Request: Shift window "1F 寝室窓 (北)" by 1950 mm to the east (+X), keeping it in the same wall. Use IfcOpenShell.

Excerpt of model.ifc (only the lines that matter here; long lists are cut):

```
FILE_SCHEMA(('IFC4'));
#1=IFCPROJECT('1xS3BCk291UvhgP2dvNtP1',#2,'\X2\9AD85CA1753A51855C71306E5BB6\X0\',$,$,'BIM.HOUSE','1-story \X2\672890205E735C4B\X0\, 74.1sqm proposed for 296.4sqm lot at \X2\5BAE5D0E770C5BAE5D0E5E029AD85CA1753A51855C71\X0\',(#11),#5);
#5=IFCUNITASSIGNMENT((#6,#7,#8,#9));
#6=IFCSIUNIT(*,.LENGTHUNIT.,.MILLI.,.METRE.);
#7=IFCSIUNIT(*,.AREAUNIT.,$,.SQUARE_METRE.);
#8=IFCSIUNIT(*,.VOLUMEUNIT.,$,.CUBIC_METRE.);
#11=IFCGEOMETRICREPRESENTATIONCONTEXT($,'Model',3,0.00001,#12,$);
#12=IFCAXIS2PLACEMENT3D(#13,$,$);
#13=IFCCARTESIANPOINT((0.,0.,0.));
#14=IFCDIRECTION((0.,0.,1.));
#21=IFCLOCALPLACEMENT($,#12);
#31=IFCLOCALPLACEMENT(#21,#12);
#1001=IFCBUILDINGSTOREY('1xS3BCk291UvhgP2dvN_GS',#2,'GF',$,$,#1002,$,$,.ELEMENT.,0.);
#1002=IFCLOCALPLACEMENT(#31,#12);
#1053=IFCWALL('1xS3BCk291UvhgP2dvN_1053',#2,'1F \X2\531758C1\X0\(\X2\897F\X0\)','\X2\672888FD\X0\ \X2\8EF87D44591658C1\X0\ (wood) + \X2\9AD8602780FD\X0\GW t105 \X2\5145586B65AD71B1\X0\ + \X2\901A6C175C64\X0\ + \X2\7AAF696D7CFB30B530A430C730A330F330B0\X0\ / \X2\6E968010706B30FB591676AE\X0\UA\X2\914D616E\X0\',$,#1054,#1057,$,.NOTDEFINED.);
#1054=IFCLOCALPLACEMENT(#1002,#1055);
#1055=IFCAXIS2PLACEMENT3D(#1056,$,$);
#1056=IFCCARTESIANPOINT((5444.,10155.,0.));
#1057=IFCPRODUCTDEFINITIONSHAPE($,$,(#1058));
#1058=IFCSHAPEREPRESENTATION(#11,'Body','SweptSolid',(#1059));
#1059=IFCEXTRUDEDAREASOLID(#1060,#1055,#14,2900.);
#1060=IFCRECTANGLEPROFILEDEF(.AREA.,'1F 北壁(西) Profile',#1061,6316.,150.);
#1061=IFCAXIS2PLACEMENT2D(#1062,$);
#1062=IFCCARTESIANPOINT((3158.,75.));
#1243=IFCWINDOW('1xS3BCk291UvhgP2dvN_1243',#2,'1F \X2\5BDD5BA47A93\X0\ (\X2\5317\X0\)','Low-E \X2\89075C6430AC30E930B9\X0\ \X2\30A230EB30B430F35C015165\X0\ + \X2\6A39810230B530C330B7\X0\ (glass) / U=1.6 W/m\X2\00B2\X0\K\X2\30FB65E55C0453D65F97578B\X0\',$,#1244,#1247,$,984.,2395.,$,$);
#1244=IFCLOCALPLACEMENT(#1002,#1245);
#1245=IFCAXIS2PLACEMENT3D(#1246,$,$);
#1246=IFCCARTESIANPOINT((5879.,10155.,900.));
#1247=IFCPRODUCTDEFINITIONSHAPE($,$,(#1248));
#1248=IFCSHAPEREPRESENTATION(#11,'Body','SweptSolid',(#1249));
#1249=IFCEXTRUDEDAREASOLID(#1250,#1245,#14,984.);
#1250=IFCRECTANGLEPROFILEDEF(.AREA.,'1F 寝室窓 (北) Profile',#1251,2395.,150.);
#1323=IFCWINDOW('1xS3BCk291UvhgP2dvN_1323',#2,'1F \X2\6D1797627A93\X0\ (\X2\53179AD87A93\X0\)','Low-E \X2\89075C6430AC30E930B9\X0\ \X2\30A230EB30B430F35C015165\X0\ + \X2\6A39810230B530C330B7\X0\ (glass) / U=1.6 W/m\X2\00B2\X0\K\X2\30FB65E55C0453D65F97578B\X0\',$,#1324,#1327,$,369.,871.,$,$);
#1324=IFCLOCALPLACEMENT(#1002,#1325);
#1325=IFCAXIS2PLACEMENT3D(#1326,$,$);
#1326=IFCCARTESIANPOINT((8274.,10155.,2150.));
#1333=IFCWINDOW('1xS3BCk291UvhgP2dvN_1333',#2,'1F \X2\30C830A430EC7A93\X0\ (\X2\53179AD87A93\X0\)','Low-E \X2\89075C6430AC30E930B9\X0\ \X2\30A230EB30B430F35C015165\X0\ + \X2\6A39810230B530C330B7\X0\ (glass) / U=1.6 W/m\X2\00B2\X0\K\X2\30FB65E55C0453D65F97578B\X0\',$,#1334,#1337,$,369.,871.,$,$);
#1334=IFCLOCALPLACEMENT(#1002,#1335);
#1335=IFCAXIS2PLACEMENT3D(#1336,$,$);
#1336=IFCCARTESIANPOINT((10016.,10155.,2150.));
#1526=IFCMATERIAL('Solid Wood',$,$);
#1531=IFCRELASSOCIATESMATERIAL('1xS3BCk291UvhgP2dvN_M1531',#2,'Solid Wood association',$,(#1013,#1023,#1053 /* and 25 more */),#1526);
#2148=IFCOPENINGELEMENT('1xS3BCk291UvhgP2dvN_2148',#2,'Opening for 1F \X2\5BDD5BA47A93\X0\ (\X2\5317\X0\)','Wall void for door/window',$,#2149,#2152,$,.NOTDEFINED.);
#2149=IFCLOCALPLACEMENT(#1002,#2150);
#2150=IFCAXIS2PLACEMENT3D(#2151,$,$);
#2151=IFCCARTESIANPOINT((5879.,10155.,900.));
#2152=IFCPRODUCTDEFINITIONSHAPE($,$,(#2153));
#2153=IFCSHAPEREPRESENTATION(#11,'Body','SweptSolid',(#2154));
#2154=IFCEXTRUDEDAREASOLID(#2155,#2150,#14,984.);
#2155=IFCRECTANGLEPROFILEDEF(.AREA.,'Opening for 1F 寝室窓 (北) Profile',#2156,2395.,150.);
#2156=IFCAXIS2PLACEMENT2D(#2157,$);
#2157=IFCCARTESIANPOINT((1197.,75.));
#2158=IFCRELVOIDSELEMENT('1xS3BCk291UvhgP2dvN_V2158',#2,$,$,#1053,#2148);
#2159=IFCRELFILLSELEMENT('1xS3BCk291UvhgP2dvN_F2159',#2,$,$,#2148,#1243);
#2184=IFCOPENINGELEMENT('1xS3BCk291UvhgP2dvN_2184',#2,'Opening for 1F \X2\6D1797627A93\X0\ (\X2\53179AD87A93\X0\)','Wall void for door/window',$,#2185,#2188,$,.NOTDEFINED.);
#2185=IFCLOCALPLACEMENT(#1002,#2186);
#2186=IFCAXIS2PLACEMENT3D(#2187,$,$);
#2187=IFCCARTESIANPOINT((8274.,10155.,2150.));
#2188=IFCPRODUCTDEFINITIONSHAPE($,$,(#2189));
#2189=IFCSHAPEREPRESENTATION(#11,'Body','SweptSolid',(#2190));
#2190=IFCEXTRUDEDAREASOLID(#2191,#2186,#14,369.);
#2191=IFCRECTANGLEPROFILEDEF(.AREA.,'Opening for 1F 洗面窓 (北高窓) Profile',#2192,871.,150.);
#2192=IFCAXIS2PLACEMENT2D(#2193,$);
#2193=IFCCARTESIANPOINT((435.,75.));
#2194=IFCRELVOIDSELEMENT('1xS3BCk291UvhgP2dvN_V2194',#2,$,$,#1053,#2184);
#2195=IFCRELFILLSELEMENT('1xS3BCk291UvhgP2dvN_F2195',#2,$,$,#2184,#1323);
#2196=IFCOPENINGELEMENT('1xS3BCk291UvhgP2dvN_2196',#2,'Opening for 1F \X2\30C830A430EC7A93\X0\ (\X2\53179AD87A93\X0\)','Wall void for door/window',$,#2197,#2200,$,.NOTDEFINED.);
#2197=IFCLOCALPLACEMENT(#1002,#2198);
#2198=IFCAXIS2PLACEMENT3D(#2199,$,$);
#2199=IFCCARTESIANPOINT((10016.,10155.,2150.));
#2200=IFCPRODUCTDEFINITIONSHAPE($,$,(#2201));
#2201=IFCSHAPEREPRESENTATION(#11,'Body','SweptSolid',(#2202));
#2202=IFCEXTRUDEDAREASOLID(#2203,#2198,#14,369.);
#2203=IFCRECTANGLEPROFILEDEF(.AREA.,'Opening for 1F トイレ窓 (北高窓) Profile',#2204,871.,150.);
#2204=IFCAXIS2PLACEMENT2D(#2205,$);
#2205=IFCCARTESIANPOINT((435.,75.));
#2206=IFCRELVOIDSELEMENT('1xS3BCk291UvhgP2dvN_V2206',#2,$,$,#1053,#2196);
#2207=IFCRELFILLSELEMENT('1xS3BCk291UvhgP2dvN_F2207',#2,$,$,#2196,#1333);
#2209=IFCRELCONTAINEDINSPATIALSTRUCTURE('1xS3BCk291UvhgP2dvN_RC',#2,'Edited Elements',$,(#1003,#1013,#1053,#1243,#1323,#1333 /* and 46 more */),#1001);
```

```python
import ifcopenshell
import ifcopenshell.api.geometry
import ifcopenshell.util.placement

model = ifcopenshell.open("model.ifc")

window = model.by_guid("1xS3BCk291UvhgP2dvN_1243")
opening = window.FillsVoids[0].RelatingOpeningElement
wall = opening.VoidsElements[0].RelatingBuildingElement

wall_matrix = ifcopenshell.util.placement.get_local_placement(wall.ObjectPlacement)
shift = wall_matrix[:3, 0] * 1950.0
before = ifcopenshell.util.placement.get_local_placement(window.ObjectPlacement)[:3, 3].copy()

# The window is not placed relative to its opening, so move both.
for product in (opening, window):
    matrix = ifcopenshell.util.placement.get_local_placement(product.ObjectPlacement)
    matrix[:3, 3] += shift
    ifcopenshell.api.geometry.edit_object_placement(model, product=product, matrix=matrix, is_si=False)

after = ifcopenshell.util.placement.get_local_placement(window.ObjectPlacement)[:3, 3]
print("window moved by", (after - before).round(3) + 0.0)

model.write("model-out.ifc")
```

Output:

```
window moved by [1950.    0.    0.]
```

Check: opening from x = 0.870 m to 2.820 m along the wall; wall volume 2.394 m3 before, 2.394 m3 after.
